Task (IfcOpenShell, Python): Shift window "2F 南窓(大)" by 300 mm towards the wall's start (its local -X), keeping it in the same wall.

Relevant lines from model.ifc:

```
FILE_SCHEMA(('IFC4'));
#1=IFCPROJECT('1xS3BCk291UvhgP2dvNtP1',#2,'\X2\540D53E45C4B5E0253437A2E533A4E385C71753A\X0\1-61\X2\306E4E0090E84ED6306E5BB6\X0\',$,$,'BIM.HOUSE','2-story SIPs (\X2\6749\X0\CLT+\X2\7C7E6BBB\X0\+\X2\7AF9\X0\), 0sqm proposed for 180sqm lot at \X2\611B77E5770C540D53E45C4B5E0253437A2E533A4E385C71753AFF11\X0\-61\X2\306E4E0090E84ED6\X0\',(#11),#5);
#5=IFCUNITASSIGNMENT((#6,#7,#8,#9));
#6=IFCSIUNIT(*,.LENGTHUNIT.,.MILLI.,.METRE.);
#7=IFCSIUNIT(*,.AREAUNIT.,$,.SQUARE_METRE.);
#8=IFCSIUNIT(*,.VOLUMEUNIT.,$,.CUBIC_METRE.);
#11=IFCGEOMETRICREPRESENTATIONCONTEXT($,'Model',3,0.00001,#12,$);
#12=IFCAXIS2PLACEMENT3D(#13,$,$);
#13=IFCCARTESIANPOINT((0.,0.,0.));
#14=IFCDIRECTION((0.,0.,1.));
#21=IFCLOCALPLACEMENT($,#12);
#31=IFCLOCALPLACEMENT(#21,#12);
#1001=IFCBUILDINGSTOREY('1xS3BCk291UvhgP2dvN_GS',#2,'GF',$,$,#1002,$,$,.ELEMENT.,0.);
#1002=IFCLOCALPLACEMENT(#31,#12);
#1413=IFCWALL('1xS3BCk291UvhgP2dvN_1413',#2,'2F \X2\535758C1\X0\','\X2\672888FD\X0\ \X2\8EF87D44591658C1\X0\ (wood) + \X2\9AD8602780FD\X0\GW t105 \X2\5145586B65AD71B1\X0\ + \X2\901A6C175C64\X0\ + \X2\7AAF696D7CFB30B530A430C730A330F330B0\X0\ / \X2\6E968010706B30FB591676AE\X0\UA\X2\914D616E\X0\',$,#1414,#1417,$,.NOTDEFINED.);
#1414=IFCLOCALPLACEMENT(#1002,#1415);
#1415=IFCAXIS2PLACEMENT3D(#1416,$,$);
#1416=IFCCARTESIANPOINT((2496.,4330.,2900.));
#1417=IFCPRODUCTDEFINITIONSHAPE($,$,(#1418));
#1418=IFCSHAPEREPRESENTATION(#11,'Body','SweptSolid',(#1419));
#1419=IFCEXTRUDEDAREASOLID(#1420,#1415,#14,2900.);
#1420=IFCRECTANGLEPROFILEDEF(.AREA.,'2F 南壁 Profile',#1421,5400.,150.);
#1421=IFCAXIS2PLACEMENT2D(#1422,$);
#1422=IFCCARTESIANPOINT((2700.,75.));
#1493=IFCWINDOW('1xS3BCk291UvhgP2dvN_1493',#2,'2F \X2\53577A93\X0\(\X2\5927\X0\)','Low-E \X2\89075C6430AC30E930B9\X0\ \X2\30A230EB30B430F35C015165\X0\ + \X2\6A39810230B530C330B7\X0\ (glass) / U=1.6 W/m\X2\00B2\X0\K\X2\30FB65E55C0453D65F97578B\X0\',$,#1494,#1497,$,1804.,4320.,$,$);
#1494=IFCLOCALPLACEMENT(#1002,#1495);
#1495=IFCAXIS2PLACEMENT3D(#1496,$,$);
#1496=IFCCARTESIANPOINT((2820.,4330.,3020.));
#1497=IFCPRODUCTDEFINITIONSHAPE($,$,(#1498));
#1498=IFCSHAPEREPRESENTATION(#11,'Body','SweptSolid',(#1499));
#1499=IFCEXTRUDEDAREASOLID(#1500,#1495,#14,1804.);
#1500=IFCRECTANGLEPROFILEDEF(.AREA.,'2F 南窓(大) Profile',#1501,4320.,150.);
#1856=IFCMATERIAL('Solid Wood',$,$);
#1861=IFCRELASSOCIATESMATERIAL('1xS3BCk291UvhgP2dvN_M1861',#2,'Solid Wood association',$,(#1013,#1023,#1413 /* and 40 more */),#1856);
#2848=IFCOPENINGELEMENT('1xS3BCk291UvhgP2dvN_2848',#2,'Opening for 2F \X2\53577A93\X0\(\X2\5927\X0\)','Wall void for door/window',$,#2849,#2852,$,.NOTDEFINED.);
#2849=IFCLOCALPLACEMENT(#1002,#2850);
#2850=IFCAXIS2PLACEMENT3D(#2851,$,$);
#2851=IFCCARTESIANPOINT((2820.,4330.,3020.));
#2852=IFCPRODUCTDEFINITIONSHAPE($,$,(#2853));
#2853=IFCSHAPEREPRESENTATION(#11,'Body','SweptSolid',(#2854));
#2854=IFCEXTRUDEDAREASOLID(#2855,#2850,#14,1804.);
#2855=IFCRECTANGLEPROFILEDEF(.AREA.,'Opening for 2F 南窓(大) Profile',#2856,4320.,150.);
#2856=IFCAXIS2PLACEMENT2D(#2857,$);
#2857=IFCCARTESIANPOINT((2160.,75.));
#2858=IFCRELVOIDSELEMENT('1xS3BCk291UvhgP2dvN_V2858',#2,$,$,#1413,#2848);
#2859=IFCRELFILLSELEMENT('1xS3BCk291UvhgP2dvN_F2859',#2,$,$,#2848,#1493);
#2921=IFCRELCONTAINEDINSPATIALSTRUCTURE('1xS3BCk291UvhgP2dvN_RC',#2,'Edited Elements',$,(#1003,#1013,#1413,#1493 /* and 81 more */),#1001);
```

```python
import ifcopenshell
import ifcopenshell.api.geometry
import ifcopenshell.util.placement
import ifcopenshell.util.unit

model = ifcopenshell.open("model.ifc")
unit_scale = ifcopenshell.util.unit.calculate_unit_scale(model)

window = model.by_guid("1xS3BCk291UvhgP2dvN_1493")
opening = window.FillsVoids[0].RelatingOpeningElement
wall = opening.VoidsElements[0].RelatingBuildingElement

wall_matrix = ifcopenshell.util.placement.get_local_placement(wall.ObjectPlacement)
shift = wall_matrix[:3, 0] * -0.3 / unit_scale
before = ifcopenshell.util.placement.get_local_placement(window.ObjectPlacement)[:3, 3].copy()

# The window is not placed relative to its opening, so move both.
for product in (opening, window):
    matrix = ifcopenshell.util.placement.get_local_placement(product.ObjectPlacement)
    matrix[:3, 3] += shift
    ifcopenshell.api.geometry.edit_object_placement(model, product=product, matrix=matrix, is_si=False)

after = ifcopenshell.util.placement.get_local_placement(window.ObjectPlacement)[:3, 3]
print("window moved by", (after - before).round(3) + 0.0)

model.write("model_v2.ifc")
```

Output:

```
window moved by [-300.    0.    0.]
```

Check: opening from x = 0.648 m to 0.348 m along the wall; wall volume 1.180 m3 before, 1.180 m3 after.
